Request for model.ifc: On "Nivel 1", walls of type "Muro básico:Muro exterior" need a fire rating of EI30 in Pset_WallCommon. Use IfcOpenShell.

First a look at what the model holds.

```python
import ifcopenshell
import ifcopenshell.util.element

model = ifcopenshell.open("model.ifc")
print(model.schema)
storey = next(s for s in model.by_type("IfcBuildingStorey") if s.Name == "Nivel 1")
walls = [e for e in ifcopenshell.util.element.get_decomposition(storey) if e.is_a("IfcWall")]
seen = {}
for e in walls:
    element_type = ifcopenshell.util.element.get_type(e)
    key = (element_type.Name if element_type != e and element_type else None, ifcopenshell.util.element.get_pset(e, "Pset_WallCommon", "FireRating"))
    seen[key] = seen.get(key, 0) + 1
for (name, value), count in sorted(seen.items(), key=str):
    print(count, "x", name, "|", value)
```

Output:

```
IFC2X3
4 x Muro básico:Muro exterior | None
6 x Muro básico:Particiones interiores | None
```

```python
import ifcopenshell
import ifcopenshell.api.pset
import ifcopenshell.util.element

model = ifcopenshell.open("model.ifc")

storey = next(s for s in model.by_type("IfcBuildingStorey") if s.Name == "Nivel 1")
walls = [e for e in ifcopenshell.util.element.get_decomposition(storey) if e.is_a("IfcWall")]

count = 0
for e in walls:
    element_type = ifcopenshell.util.element.get_type(e)
    if element_type in (None, e) or element_type.Name != "Muro básico:Muro exterior":
        continue
    # add_pset returns the element's existing set when there is one.
    pset = ifcopenshell.api.pset.add_pset(model, product=e, name="Pset_WallCommon")
    ifcopenshell.api.pset.edit_pset(model, pset=pset, properties={"FireRating": "EI30"})
    count += 1

print(count, "walls updated")

model.write("model-out.ifc")
```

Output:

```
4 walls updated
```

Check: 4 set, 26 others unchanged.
